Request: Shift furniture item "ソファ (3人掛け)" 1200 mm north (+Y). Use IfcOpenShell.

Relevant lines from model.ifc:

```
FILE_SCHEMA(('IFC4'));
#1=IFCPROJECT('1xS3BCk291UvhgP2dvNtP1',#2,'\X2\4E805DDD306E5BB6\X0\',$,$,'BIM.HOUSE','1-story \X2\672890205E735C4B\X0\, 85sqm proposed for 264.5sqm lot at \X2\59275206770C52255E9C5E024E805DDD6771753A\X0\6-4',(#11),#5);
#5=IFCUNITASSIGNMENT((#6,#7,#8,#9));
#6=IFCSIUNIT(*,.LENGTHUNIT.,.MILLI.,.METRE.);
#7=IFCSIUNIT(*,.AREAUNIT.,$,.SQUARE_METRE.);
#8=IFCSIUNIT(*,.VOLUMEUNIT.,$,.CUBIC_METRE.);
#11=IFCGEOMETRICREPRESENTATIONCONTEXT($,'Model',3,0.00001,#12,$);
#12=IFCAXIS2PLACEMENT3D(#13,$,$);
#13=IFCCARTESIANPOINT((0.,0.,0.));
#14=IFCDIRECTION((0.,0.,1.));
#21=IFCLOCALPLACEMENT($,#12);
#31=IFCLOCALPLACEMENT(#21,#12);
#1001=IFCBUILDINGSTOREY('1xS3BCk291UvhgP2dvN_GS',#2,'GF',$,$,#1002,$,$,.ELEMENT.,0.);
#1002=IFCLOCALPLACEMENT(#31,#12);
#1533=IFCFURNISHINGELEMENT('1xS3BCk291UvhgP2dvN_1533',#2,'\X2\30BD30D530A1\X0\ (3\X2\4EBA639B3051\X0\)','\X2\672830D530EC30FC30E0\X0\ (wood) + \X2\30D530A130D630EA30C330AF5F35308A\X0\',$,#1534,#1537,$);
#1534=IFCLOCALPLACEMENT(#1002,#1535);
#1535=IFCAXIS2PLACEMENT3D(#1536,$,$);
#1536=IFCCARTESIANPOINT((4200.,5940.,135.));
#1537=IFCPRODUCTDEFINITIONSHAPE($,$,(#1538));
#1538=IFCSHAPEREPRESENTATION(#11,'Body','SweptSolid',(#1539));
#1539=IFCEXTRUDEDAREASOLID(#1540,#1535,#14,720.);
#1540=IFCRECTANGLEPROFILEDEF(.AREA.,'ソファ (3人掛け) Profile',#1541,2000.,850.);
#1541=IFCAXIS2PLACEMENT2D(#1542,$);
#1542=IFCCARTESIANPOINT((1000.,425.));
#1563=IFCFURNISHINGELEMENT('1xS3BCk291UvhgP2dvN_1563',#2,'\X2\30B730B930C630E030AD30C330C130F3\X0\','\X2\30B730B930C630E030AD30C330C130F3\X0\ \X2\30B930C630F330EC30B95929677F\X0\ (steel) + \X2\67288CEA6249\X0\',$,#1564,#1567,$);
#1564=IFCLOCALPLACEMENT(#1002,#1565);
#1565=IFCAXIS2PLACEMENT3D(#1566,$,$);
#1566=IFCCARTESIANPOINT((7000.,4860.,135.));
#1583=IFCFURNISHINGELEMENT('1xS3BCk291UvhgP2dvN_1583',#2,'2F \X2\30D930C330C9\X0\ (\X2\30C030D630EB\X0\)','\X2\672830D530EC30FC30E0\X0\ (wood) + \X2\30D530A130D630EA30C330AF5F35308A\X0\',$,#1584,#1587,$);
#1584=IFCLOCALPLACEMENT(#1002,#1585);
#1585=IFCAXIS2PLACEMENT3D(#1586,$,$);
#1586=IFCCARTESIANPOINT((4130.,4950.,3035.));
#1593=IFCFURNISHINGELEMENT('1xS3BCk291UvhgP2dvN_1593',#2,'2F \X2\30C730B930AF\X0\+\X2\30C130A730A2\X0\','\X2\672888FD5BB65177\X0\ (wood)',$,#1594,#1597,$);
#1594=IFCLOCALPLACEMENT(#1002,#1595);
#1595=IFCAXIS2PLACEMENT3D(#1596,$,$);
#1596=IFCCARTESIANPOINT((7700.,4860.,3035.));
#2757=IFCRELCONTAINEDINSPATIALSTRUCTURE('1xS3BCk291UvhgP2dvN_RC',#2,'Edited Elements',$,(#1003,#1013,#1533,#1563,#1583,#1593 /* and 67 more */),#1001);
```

```python
import ifcopenshell
import ifcopenshell.api.geometry
import ifcopenshell.util.placement

model = ifcopenshell.open("model.ifc")

item = model.by_guid("1xS3BCk291UvhgP2dvN_1533")
matrix = ifcopenshell.util.placement.get_local_placement(item.ObjectPlacement)
matrix[1, 3] += 1200.0
ifcopenshell.api.geometry.edit_object_placement(model, product=item, matrix=matrix, is_si=False)

print(ifcopenshell.util.placement.get_local_placement(item.ObjectPlacement).round(3) + 0.0)

model.write("model_v2.ifc")
```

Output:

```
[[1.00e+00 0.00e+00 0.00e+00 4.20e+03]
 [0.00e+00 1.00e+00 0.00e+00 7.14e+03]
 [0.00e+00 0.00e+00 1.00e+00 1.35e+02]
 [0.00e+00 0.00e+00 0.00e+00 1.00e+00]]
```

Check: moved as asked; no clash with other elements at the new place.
